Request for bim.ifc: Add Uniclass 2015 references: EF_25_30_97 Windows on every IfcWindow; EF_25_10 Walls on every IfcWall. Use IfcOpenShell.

First a look at what the model holds.

```python
import ifcopenshell

model = ifcopenshell.open("bim.ifc")
print(model.schema)
print("classifications:", [c.Name for c in model.by_type("IfcClassification")])
for ifc_class in ("IfcDoor", "IfcRoof", "IfcStair", "IfcWall", "IfcWindow"):
    print(ifc_class, len(model.by_type(ifc_class)))
```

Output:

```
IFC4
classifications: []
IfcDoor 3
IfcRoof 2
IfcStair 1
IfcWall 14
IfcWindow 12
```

```python
import ifcopenshell
import ifcopenshell.api.classification

model = ifcopenshell.open("bim.ifc")

system = ifcopenshell.api.classification.add_classification(model, classification="Uniclass 2015")

codes = {
    "IfcWindow": ("EF_25_30_97", "Windows"),
    "IfcWall": ("EF_25_10", "Walls"),
}
for ifc_class, (code, name) in codes.items():
    products = model.by_type(ifc_class)
    ifcopenshell.api.classification.add_reference(
        model, products=products, classification=system, identification=code, name=name
    )
    print(code, len(products))

model.write("bim_rev.ifc")
```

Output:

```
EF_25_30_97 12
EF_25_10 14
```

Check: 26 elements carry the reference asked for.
